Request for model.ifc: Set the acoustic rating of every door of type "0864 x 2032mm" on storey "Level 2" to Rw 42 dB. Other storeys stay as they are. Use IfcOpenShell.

First a look at what the model holds.

```python
import ifcopenshell
import ifcopenshell.util.element

model = ifcopenshell.open("model.ifc")
print(model.schema)
storey = next(s for s in model.by_type("IfcBuildingStorey") if s.Name == "Level 2")
doors = [e for e in ifcopenshell.util.element.get_decomposition(storey) if e.is_a("IfcDoor")]
seen = {}
for e in doors:
    element_type = ifcopenshell.util.element.get_type(e)
    key = (element_type.Name if element_type != e and element_type else None, ifcopenshell.util.element.get_pset(e, "Pset_DoorCommon", "AcousticRating"))
    seen[key] = seen.get(key, 0) + 1
for (name, value), count in sorted(seen.items(), key=str):
    print(count, "x", name, "|", value)
```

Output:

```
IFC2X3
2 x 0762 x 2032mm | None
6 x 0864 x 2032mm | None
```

```python
import ifcopenshell
import ifcopenshell.api.pset
import ifcopenshell.util.element

model = ifcopenshell.open("model.ifc")

storey = next(s for s in model.by_type("IfcBuildingStorey") if s.Name == "Level 2")
doors = [e for e in ifcopenshell.util.element.get_decomposition(storey) if e.is_a("IfcDoor")]

count = 0
for e in doors:
    element_type = ifcopenshell.util.element.get_type(e)
    if element_type in (None, e) or element_type.Name != "0864 x 2032mm":
        continue
    # add_pset returns the element's existing set when there is one.
    pset = ifcopenshell.api.pset.add_pset(model, product=e, name="Pset_DoorCommon")
    ifcopenshell.api.pset.edit_pset(model, pset=pset, properties={"AcousticRating": "Rw 42 dB"})
    count += 1

print(count, "doors updated")

model.write("model_v2.ifc")
```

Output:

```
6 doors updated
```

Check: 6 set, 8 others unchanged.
